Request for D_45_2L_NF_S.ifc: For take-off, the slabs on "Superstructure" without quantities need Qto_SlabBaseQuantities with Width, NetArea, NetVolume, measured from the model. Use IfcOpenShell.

First a look at what the model holds.

```python
import ifcopenshell
import ifcopenshell.util.element
import ifcopenshell.util.unit

model = ifcopenshell.open("D_45_2L_NF_S.ifc")
print(model.schema)
for unit_type in ("LENGTHUNIT", "AREAUNIT", "VOLUMEUNIT"):
    print(unit_type, ifcopenshell.util.unit.calculate_unit_scale(model, unit_type))
storey = next(s for s in model.by_type("IfcBuildingStorey") if s.Name == "Superstructure")
slabs = [e for e in ifcopenshell.util.element.get_decomposition(storey) if e.is_a("IfcSlab")]
for e in sorted(slabs, key=lambda e: e.id()):
    print(e.id(), e.is_a(), e.Name, list(ifcopenshell.util.element.get_psets(e, qtos_only=True)), sep=" | ")
```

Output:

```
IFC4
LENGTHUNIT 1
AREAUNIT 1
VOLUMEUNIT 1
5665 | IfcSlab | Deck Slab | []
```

```python
import ifcopenshell
import ifcopenshell.api.pset
import ifcopenshell.geom
import ifcopenshell.util.element
import ifcopenshell.util.shape
import ifcopenshell.util.unit

model = ifcopenshell.open("D_45_2L_NF_S.ifc")
unit_scale = ifcopenshell.util.unit.calculate_unit_scale(model)
area_scale = ifcopenshell.util.unit.calculate_unit_scale(model, "AREAUNIT")
volume_scale = ifcopenshell.util.unit.calculate_unit_scale(model, "VOLUMEUNIT")
settings = ifcopenshell.geom.settings()

storey = next(s for s in model.by_type("IfcBuildingStorey") if s.Name == "Superstructure")
slabs = [e for e in ifcopenshell.util.element.get_decomposition(storey) if e.is_a("IfcSlab")]

for e in sorted(slabs, key=lambda e: e.id()):
    if ifcopenshell.util.element.get_psets(e, qtos_only=True, should_inherit=False):
        continue
    # Geometry comes back in metres, in the element's own axes.
    shape = ifcopenshell.geom.create_shape(settings, e)
    values = {
        "Width": ifcopenshell.util.shape.get_z(shape.geometry) / unit_scale,
        "NetArea": ifcopenshell.util.shape.get_footprint_area(shape.geometry) / area_scale,
        "NetVolume": ifcopenshell.util.shape.get_volume(shape.geometry) / volume_scale,
    }
    qto = ifcopenshell.api.pset.add_qto(model, product=e, name="Qto_SlabBaseQuantities")
    ifcopenshell.api.pset.edit_qto(model, qto=qto, properties=values)
    print(e.id(), {k: round(v, 3) for k, v in values.items()})

model.write("D_45_2L_NF_S-out.ifc")
```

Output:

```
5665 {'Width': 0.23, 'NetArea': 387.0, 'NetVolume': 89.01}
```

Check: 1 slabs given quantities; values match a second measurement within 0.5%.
